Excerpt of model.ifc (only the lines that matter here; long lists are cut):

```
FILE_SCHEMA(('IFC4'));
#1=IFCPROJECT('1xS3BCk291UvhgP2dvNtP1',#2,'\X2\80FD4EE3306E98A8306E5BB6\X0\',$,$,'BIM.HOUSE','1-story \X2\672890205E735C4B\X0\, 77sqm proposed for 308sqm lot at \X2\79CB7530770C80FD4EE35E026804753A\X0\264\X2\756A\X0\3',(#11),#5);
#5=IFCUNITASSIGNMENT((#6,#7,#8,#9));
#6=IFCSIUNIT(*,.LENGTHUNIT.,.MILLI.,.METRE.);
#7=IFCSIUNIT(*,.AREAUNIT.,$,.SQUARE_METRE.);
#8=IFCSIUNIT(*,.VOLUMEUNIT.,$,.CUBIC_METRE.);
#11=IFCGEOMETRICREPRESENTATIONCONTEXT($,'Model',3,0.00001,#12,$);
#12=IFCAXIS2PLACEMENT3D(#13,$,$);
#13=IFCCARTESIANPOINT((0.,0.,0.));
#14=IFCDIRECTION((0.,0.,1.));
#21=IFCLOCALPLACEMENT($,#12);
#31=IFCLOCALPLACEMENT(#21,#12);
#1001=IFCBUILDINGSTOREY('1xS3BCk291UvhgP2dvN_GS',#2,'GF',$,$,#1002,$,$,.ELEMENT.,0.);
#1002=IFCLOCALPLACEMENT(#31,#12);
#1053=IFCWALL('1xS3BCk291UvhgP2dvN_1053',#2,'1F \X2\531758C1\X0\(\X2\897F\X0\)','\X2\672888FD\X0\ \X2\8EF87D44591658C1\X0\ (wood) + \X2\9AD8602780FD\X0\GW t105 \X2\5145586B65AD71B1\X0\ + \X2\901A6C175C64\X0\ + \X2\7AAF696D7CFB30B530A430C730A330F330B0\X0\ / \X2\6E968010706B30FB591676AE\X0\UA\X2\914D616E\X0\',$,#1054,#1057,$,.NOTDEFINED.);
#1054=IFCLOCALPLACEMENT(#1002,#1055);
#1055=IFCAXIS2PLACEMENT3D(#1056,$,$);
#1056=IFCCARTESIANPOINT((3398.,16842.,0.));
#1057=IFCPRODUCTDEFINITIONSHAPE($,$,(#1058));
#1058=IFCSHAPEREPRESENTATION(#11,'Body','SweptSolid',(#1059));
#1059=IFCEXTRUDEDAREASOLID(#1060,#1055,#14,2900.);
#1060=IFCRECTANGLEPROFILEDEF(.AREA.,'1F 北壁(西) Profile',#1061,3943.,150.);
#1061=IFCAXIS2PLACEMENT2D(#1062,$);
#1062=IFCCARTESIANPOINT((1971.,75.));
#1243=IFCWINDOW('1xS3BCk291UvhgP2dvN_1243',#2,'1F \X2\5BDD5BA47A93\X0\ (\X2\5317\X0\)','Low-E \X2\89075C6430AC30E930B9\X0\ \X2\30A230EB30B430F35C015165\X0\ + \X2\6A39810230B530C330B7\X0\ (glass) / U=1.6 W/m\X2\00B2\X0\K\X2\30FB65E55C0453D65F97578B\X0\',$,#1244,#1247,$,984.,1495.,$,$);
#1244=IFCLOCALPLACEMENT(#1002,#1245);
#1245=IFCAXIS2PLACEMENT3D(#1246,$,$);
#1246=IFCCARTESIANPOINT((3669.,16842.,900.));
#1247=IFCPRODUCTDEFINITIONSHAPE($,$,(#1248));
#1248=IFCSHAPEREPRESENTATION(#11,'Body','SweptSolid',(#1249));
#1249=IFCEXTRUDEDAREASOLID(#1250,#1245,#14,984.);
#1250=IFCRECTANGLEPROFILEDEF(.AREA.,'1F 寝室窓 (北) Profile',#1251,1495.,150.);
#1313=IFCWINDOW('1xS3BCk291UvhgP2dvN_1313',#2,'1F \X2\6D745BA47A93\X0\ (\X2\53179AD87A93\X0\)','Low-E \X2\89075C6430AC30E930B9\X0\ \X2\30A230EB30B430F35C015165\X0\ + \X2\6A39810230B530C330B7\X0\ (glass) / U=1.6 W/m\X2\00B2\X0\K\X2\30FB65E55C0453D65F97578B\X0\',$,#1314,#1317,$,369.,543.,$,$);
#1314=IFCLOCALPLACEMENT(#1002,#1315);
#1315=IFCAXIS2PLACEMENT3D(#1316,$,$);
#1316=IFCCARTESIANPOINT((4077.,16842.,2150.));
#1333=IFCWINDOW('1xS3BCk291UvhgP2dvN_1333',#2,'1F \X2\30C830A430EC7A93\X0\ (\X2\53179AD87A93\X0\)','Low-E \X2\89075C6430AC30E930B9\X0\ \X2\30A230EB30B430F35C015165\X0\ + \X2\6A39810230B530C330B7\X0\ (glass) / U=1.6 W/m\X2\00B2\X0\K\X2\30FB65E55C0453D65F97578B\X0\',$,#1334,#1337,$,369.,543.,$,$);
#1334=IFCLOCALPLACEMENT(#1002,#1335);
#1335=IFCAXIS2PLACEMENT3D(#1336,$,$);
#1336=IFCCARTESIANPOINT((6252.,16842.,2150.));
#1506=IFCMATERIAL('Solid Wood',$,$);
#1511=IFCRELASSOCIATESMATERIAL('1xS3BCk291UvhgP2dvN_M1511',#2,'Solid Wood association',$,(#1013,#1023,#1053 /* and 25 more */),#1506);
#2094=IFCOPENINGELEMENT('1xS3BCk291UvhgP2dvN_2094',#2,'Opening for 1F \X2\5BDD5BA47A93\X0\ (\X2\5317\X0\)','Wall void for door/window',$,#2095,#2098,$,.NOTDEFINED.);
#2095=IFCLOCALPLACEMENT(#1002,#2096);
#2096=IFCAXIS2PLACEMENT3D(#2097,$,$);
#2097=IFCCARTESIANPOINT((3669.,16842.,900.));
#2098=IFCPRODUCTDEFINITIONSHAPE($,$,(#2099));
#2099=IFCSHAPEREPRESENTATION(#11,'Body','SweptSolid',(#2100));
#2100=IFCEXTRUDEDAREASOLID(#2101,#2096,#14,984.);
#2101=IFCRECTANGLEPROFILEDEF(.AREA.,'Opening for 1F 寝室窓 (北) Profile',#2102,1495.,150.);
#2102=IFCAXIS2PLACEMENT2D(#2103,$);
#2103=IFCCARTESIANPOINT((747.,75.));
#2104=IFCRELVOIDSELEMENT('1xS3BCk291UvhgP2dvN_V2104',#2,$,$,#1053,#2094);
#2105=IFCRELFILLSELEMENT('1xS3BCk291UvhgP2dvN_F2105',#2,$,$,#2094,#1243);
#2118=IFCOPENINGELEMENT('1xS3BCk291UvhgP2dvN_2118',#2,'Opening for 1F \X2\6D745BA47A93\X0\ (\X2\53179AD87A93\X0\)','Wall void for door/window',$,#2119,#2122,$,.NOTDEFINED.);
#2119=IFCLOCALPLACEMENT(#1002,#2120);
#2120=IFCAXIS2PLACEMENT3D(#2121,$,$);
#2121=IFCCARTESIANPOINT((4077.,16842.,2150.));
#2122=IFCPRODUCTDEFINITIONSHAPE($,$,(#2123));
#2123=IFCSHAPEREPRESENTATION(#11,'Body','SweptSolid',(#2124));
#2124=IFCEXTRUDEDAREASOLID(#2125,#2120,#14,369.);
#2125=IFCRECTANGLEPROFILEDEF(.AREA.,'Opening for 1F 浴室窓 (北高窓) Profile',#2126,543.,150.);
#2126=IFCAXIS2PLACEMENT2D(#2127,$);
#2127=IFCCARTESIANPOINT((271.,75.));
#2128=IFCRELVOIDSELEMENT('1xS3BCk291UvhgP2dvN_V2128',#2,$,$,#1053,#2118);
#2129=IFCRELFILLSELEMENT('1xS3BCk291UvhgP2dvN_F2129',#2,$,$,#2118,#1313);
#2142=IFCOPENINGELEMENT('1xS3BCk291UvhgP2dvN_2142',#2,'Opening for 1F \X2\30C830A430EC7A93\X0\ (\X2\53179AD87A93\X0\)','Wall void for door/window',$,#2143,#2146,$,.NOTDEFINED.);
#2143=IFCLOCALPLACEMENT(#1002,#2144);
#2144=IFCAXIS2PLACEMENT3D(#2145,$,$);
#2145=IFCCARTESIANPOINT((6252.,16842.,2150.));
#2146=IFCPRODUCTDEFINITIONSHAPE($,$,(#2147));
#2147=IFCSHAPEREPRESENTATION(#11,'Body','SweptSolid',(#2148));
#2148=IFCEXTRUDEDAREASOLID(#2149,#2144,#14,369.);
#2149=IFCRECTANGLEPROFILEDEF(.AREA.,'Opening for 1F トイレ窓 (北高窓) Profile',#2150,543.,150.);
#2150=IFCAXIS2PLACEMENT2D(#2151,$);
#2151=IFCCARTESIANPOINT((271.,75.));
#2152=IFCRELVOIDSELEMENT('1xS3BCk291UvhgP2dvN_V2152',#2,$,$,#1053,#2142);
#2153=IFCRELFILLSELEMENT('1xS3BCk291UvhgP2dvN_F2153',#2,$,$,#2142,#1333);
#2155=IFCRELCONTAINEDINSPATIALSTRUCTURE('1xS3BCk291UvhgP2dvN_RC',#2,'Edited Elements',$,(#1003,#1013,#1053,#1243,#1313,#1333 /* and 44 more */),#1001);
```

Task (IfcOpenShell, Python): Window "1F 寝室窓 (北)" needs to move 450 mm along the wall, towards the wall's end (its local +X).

```python
import ifcopenshell
import ifcopenshell.api.geometry
import ifcopenshell.util.placement

model = ifcopenshell.open("model.ifc")

window = model.by_guid("1xS3BCk291UvhgP2dvN_1243")
opening = window.FillsVoids[0].RelatingOpeningElement
wall = opening.VoidsElements[0].RelatingBuildingElement

wall_matrix = ifcopenshell.util.placement.get_local_placement(wall.ObjectPlacement)
shift = wall_matrix[:3, 0] * 450.0
before = ifcopenshell.util.placement.get_local_placement(window.ObjectPlacement)[:3, 3].copy()

# The window is not placed relative to its opening, so move both.
for product in (opening, window):
    matrix = ifcopenshell.util.placement.get_local_placement(product.ObjectPlacement)
    matrix[:3, 3] += shift
    ifcopenshell.api.geometry.edit_object_placement(model, product=product, matrix=matrix, is_si=False)

after = ifcopenshell.util.placement.get_local_placement(window.ObjectPlacement)[:3, 3]
print("window moved by", (after - before).round(3) + 0.0)

model.write("model_v2.ifc")
```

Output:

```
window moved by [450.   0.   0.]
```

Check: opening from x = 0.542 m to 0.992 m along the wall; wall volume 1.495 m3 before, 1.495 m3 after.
